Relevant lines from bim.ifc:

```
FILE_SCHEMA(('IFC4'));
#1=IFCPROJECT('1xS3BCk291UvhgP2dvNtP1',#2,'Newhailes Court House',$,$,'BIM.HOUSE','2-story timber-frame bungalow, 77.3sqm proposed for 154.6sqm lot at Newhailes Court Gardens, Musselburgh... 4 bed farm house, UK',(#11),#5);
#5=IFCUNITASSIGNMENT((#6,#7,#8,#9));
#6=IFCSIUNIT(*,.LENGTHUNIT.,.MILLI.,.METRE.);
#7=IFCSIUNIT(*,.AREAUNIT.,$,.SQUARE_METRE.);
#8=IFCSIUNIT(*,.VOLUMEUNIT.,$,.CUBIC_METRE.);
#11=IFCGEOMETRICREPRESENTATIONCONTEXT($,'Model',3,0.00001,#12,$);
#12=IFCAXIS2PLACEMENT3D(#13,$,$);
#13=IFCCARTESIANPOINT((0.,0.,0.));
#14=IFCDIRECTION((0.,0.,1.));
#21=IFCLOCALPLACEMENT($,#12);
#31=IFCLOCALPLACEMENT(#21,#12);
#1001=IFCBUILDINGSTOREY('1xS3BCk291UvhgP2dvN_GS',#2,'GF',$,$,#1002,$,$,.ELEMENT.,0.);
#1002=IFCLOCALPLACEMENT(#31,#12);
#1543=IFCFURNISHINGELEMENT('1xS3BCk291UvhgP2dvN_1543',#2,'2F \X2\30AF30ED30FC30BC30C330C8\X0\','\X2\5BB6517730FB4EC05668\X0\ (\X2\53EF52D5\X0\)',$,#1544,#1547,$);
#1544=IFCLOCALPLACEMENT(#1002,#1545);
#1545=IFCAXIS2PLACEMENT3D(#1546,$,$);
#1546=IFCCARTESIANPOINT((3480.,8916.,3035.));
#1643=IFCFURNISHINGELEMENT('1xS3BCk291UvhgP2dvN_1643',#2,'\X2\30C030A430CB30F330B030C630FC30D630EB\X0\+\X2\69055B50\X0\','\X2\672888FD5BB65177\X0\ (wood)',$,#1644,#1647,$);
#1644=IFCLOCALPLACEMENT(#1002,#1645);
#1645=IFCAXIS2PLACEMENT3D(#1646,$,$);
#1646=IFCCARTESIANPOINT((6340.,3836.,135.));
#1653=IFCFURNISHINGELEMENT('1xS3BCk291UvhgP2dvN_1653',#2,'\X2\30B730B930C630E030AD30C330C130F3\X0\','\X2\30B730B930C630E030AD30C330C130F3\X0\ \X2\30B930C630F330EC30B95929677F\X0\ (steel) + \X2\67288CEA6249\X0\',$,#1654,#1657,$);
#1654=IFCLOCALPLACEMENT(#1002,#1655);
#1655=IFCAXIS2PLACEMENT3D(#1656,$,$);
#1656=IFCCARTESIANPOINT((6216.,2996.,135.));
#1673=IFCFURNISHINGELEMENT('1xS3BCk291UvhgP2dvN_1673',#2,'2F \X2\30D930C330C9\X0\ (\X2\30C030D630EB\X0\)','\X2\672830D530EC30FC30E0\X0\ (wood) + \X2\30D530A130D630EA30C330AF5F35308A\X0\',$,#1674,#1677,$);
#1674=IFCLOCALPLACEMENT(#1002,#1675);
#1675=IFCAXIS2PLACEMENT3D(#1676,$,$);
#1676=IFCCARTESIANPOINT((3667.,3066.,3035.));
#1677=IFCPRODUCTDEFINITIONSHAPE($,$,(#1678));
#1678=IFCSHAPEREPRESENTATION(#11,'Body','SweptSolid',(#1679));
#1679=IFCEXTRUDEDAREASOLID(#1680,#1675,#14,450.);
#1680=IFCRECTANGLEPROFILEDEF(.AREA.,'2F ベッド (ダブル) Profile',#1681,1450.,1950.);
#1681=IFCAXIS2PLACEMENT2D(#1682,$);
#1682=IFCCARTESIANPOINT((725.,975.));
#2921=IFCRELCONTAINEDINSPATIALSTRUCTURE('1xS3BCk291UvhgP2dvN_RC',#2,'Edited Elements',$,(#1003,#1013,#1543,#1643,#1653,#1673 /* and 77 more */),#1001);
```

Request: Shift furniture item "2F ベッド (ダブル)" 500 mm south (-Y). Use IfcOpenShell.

```python
import ifcopenshell
import ifcopenshell.api.geometry
import ifcopenshell.util.placement
import ifcopenshell.util.unit

model = ifcopenshell.open("bim.ifc")
unit_scale = ifcopenshell.util.unit.calculate_unit_scale(model)

item = model.by_guid("1xS3BCk291UvhgP2dvN_1673")
matrix = ifcopenshell.util.placement.get_local_placement(item.ObjectPlacement)
matrix[1, 3] -= 0.5 / unit_scale
ifcopenshell.api.geometry.edit_object_placement(model, product=item, matrix=matrix, is_si=False)

print(ifcopenshell.util.placement.get_local_placement(item.ObjectPlacement).round(3) + 0.0)

model.write("bim_edited.ifc")
```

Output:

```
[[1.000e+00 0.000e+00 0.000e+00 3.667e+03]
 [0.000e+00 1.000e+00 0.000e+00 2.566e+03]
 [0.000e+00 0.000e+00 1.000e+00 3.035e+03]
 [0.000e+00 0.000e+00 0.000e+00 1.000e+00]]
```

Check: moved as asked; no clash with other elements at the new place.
